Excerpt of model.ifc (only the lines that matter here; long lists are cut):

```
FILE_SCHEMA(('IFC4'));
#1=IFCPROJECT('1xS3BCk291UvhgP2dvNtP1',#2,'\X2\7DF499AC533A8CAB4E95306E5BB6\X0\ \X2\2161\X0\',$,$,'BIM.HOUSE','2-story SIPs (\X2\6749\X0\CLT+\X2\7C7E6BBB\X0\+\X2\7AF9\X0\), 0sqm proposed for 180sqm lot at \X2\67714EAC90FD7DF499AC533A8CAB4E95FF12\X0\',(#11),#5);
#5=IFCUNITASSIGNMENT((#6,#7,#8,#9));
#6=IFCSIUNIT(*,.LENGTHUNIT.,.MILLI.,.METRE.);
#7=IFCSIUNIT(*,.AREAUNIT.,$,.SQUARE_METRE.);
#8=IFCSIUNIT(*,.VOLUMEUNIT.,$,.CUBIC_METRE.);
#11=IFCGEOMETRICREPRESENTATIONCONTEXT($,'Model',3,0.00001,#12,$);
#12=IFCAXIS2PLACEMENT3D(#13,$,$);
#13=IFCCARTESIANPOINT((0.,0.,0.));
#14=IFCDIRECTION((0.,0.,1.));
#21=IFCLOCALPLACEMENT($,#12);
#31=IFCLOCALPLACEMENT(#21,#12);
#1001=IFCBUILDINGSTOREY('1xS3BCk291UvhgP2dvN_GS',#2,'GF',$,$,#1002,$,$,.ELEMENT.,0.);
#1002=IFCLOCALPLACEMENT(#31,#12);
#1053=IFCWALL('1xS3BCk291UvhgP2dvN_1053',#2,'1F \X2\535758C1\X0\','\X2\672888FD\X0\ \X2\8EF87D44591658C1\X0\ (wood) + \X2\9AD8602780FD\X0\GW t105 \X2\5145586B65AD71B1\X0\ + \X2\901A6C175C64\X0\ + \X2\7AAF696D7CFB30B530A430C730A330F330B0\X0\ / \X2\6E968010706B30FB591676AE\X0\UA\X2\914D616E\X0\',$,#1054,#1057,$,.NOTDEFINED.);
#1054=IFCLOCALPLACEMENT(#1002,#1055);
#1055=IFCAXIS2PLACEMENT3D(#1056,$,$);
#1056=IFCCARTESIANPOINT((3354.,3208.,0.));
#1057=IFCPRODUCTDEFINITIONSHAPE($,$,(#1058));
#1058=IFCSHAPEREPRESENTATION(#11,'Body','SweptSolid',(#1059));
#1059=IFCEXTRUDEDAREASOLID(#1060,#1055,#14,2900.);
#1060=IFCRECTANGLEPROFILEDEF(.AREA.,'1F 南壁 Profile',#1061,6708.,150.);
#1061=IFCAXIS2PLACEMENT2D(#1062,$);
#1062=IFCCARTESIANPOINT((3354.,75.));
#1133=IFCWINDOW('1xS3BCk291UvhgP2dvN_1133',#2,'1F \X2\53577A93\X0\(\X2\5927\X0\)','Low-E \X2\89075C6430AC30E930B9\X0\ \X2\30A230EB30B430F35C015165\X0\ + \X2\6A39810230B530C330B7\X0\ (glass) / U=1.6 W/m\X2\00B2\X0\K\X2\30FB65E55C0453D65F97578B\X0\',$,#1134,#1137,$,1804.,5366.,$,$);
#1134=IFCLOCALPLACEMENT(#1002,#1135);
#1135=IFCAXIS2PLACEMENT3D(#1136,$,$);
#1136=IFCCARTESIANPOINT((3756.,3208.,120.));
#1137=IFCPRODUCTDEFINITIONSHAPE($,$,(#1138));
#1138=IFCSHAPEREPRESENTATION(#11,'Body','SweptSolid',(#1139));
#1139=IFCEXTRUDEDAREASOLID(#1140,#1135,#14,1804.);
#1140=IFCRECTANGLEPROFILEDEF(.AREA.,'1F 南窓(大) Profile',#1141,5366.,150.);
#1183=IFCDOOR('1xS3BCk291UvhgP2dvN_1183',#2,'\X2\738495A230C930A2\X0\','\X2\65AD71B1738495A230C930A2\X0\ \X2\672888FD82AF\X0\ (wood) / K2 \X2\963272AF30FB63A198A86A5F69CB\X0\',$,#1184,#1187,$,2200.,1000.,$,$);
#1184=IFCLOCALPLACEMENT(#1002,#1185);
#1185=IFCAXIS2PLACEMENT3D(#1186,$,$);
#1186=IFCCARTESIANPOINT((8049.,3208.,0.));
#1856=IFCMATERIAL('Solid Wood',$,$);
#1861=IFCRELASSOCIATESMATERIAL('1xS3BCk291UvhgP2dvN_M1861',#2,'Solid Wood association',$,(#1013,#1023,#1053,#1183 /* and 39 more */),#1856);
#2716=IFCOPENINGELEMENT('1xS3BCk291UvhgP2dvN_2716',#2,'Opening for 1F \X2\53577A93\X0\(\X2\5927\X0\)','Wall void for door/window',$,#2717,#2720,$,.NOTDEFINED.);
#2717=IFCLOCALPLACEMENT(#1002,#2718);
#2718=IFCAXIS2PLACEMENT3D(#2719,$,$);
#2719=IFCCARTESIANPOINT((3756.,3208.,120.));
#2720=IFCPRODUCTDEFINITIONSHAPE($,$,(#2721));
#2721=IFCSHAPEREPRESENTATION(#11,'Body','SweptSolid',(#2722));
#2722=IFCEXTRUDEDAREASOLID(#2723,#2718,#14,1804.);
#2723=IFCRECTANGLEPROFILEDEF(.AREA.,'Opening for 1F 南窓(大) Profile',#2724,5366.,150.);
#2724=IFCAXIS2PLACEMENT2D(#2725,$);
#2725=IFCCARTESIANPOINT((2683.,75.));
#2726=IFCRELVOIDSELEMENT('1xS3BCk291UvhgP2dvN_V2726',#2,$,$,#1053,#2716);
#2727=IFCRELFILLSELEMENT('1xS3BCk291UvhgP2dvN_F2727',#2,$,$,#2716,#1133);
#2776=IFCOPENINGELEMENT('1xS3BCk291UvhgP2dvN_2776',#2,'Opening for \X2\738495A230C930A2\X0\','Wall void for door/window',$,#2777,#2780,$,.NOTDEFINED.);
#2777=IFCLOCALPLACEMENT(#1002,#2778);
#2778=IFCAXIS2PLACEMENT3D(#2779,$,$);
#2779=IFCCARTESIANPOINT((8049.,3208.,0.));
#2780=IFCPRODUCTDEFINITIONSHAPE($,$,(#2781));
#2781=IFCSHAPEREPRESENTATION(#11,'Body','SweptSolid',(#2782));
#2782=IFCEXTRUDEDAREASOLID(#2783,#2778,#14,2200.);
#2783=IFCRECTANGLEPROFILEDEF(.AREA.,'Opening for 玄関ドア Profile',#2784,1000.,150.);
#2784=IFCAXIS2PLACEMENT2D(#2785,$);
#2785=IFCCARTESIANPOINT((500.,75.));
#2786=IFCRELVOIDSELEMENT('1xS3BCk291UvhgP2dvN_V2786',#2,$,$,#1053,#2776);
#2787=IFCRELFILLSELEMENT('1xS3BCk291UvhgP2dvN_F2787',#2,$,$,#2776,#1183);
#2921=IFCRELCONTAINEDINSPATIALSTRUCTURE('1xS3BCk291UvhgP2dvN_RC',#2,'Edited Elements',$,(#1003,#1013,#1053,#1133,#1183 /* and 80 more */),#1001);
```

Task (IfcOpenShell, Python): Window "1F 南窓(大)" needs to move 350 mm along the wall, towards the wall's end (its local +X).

```python
import ifcopenshell
import ifcopenshell.api.geometry
import ifcopenshell.util.placement
import ifcopenshell.util.unit

model = ifcopenshell.open("model.ifc")
unit_scale = ifcopenshell.util.unit.calculate_unit_scale(model)

window = model.by_guid("1xS3BCk291UvhgP2dvN_1133")
opening = window.FillsVoids[0].RelatingOpeningElement
wall = opening.VoidsElements[0].RelatingBuildingElement

wall_matrix = ifcopenshell.util.placement.get_local_placement(wall.ObjectPlacement)
shift = wall_matrix[:3, 0] * 0.35 / unit_scale
before = ifcopenshell.util.placement.get_local_placement(window.ObjectPlacement)[:3, 3].copy()

# The window is not placed relative to its opening, so move both.
for product in (opening, window):
    matrix = ifcopenshell.util.placement.get_local_placement(product.ObjectPlacement)
    matrix[:3, 3] += shift
    ifcopenshell.api.geometry.edit_object_placement(model, product=product, matrix=matrix, is_si=False)

after = ifcopenshell.util.placement.get_local_placement(window.ObjectPlacement)[:3, 3]
print("window moved by", (after - before).round(3) + 0.0)

model.write("model_v2.ifc")
```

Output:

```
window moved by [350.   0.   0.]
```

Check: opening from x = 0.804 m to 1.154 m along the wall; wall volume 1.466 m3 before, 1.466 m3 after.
